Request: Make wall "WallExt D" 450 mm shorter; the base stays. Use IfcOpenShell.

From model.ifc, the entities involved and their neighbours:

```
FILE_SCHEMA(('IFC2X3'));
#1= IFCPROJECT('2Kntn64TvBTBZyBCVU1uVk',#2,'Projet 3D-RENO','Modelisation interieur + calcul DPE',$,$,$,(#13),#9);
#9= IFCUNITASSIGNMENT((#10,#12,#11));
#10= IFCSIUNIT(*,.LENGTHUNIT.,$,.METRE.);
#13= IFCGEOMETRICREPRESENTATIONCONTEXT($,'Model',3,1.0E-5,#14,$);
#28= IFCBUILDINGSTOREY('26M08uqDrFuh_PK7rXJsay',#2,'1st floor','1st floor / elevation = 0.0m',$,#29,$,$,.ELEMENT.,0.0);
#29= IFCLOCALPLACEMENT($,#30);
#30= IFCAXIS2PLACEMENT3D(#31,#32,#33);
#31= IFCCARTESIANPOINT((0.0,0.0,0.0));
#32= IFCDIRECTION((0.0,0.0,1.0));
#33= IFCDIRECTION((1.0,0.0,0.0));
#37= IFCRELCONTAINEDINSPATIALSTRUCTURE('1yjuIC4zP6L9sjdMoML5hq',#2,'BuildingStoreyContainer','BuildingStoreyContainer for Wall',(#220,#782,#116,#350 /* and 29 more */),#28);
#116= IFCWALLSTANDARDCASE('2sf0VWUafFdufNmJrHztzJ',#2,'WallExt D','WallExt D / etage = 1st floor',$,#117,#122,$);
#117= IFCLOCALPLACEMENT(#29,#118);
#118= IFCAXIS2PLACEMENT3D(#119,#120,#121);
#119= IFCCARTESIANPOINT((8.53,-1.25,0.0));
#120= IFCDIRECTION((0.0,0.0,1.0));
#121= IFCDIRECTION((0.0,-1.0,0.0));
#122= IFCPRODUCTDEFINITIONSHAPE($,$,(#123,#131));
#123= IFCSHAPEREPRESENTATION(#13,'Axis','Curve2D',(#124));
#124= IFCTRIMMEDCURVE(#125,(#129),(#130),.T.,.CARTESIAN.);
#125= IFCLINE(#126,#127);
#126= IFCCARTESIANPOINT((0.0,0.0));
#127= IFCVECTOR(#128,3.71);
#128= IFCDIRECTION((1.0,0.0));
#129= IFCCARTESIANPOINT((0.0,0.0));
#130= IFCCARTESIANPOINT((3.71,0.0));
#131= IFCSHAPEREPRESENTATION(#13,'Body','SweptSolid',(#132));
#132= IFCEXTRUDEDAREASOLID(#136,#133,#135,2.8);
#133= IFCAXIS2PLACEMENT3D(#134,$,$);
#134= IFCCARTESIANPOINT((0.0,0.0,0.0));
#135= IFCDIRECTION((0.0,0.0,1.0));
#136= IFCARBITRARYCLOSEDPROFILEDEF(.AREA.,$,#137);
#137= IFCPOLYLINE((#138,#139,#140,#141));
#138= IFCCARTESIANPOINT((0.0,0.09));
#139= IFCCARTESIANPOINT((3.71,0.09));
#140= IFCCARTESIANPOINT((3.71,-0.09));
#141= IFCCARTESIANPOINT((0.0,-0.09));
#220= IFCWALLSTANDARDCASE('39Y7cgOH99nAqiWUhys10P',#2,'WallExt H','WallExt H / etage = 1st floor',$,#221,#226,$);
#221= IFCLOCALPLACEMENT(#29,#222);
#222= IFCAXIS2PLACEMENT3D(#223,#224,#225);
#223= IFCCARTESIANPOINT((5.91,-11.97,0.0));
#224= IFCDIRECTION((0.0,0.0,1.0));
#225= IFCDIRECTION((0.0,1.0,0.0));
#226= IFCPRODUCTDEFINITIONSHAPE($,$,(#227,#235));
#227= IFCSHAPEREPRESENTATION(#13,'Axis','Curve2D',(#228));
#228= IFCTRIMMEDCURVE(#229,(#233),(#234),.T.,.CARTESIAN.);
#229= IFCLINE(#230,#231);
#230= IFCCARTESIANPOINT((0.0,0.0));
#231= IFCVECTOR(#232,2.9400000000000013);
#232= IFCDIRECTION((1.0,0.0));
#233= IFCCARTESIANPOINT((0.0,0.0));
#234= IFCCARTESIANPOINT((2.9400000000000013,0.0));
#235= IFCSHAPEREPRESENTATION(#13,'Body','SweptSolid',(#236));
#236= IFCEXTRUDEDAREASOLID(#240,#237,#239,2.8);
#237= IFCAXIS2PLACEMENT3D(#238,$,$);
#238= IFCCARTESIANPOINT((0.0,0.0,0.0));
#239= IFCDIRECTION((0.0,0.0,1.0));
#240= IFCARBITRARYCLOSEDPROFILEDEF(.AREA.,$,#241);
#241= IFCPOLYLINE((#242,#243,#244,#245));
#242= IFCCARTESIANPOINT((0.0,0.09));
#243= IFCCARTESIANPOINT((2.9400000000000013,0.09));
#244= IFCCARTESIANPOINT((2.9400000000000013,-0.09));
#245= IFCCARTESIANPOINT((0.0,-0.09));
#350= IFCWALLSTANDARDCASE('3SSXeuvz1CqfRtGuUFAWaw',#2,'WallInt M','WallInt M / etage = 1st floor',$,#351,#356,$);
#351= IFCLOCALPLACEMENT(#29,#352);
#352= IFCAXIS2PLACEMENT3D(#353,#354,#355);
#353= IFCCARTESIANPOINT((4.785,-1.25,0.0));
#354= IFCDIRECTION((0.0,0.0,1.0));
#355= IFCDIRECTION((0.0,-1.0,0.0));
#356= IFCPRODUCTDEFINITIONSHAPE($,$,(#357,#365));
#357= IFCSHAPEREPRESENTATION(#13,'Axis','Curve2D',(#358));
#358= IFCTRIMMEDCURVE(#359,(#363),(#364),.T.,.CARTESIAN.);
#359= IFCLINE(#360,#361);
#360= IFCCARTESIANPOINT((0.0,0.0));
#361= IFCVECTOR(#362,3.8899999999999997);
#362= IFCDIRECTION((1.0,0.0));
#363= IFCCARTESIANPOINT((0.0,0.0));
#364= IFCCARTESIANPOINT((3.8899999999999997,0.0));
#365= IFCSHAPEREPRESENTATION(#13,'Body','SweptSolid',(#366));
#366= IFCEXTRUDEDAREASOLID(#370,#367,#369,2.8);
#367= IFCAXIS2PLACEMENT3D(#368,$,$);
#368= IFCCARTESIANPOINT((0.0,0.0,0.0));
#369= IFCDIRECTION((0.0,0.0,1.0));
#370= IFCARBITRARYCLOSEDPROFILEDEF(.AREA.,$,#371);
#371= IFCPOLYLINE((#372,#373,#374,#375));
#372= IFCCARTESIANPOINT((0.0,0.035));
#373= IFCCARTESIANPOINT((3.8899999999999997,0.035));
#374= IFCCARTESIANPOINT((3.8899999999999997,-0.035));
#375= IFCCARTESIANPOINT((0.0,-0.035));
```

```python
import ifcopenshell
import ifcopenshell.geom
import ifcopenshell.util.shape
import ifcopenshell.util.unit

model = ifcopenshell.open("model.ifc")
unit_scale = ifcopenshell.util.unit.calculate_unit_scale(model)
settings = ifcopenshell.geom.settings()


def volume(element):
    """Net volume in cubic metres, openings subtracted."""
    shape = ifcopenshell.geom.create_shape(settings, element)
    return ifcopenshell.util.shape.get_volume(shape.geometry)


wall = model.by_guid("2sf0VWUafFdufNmJrHztzJ")
before = volume(wall)

body = next(r for r in wall.Representation.Representations if r.RepresentationIdentifier == "Body")
solid = body.Items[0]
old_height = solid.Depth
solid.Depth -= 0.45 / unit_scale
after = volume(wall)

print(f"height {old_height:g} -> {solid.Depth:g}, volume {before:.3f} -> {after:.3f} m3")

model.write("model_edited.ifc")
```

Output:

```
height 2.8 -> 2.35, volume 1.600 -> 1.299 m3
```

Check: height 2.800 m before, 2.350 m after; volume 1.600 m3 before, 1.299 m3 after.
